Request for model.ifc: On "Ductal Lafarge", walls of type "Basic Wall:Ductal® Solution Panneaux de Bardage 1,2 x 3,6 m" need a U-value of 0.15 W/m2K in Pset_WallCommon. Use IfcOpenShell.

First a look at what the model holds.

```python
import ifcopenshell
import ifcopenshell.util.element

model = ifcopenshell.open("model.ifc")
print(model.schema)
storey = next(s for s in model.by_type("IfcBuildingStorey") if s.Name == "Ductal Lafarge")
walls = [e for e in ifcopenshell.util.element.get_decomposition(storey) if e.is_a("IfcWall")]
seen = {}
for e in walls:
    element_type = ifcopenshell.util.element.get_type(e)
    key = (element_type.Name if element_type != e and element_type else None, ifcopenshell.util.element.get_pset(e, "Pset_WallCommon", "ThermalTransmittance"))
    seen[key] = seen.get(key, 0) + 1
for (name, value), count in sorted(seen.items(), key=str):
    print(count, "x", name, "|", value)
```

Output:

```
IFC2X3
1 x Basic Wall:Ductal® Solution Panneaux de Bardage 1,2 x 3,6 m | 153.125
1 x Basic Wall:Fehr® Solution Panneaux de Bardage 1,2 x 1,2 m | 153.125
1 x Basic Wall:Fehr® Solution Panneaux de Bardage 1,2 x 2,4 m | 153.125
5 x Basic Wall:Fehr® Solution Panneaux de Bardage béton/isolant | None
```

```python
import ifcopenshell
import ifcopenshell.api.pset
import ifcopenshell.util.element

model = ifcopenshell.open("model.ifc")

storey = next(s for s in model.by_type("IfcBuildingStorey") if s.Name == "Ductal Lafarge")
walls = [e for e in ifcopenshell.util.element.get_decomposition(storey) if e.is_a("IfcWall")]

count = 0
for e in walls:
    element_type = ifcopenshell.util.element.get_type(e)
    if element_type in (None, e) or element_type.Name != "Basic Wall:Ductal® Solution Panneaux de Bardage 1,2 x 3,6 m":
        continue
    # add_pset returns the element's existing set when there is one.
    pset = ifcopenshell.api.pset.add_pset(model, product=e, name="Pset_WallCommon")
    ifcopenshell.api.pset.edit_pset(model, pset=pset, properties={"ThermalTransmittance": 0.15})
    count += 1

print(count, "walls updated")

model.write("model_v2.ifc")
```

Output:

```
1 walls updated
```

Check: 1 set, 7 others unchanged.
